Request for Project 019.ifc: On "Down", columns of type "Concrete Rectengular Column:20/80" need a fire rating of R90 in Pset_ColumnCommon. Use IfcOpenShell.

First a look at what the model holds.

```python
import ifcopenshell
import ifcopenshell.util.element

model = ifcopenshell.open("Project 019.ifc")
print(model.schema)
storey = next(s for s in model.by_type("IfcBuildingStorey") if s.Name == "Down")
columns = [e for e in ifcopenshell.util.element.get_decomposition(storey) if e.is_a("IfcColumn")]
seen = {}
for e in columns:
    element_type = ifcopenshell.util.element.get_type(e)
    key = (element_type.Name if element_type != e and element_type else None, ifcopenshell.util.element.get_pset(e, "Pset_ColumnCommon", "FireRating"))
    seen[key] = seen.get(key, 0) + 1
for (name, value), count in sorted(seen.items(), key=str):
    print(count, "x", name, "|", value)
```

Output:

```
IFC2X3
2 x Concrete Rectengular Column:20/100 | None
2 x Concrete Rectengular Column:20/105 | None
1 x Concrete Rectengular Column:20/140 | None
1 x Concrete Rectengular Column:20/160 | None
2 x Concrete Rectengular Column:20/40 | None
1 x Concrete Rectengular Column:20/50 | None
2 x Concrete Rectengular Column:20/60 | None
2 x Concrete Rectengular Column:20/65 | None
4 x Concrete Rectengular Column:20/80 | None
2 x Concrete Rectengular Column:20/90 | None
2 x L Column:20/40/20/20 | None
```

```python
import ifcopenshell
import ifcopenshell.api.pset
import ifcopenshell.util.element

model = ifcopenshell.open("Project 019.ifc")

storey = next(s for s in model.by_type("IfcBuildingStorey") if s.Name == "Down")
columns = [e for e in ifcopenshell.util.element.get_decomposition(storey) if e.is_a("IfcColumn")]

count = 0
for e in columns:
    element_type = ifcopenshell.util.element.get_type(e)
    if element_type in (None, e) or element_type.Name != "Concrete Rectengular Column:20/80":
        continue
    # add_pset returns the element's existing set when there is one.
    pset = ifcopenshell.api.pset.add_pset(model, product=e, name="Pset_ColumnCommon")
    ifcopenshell.api.pset.edit_pset(model, pset=pset, properties={"FireRating": "R90"})
    count += 1

print(count, "columns updated")

model.write("Project 019-out.ifc")
```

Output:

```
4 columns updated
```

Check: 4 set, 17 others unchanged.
